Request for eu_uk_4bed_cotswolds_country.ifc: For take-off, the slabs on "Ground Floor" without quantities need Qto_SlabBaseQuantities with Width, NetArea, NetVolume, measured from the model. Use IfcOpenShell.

First a look at what the model holds.

```python
import ifcopenshell
import ifcopenshell.util.element
import ifcopenshell.util.unit

model = ifcopenshell.open("eu_uk_4bed_cotswolds_country.ifc")
print(model.schema)
for unit_type in ("LENGTHUNIT", "AREAUNIT", "VOLUMEUNIT"):
    print(unit_type, ifcopenshell.util.unit.calculate_unit_scale(model, unit_type))
storey = next(s for s in model.by_type("IfcBuildingStorey") if s.Name == "Ground Floor")
slabs = [e for e in ifcopenshell.util.element.get_decomposition(storey) if e.is_a("IfcSlab")]
for e in sorted(slabs, key=lambda e: e.id()):
    print(e.id(), e.is_a(), e.Name, list(ifcopenshell.util.element.get_psets(e, qtos_only=True)), sep=" | ")
```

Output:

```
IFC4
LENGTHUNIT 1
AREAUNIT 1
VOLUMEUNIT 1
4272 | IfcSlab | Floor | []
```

```python
import ifcopenshell
import ifcopenshell.api.pset
import ifcopenshell.geom
import ifcopenshell.util.element
import ifcopenshell.util.shape
import ifcopenshell.util.unit

model = ifcopenshell.open("eu_uk_4bed_cotswolds_country.ifc")
unit_scale = ifcopenshell.util.unit.calculate_unit_scale(model)
area_scale = ifcopenshell.util.unit.calculate_unit_scale(model, "AREAUNIT")
volume_scale = ifcopenshell.util.unit.calculate_unit_scale(model, "VOLUMEUNIT")
settings = ifcopenshell.geom.settings()

storey = next(s for s in model.by_type("IfcBuildingStorey") if s.Name == "Ground Floor")
slabs = [e for e in ifcopenshell.util.element.get_decomposition(storey) if e.is_a("IfcSlab")]

for e in sorted(slabs, key=lambda e: e.id()):
    if ifcopenshell.util.element.get_psets(e, qtos_only=True, should_inherit=False):
        continue
    # Geometry comes back in metres, in the element's own axes.
    shape = ifcopenshell.geom.create_shape(settings, e)
    values = {
        "Width": ifcopenshell.util.shape.get_z(shape.geometry) / unit_scale,
        "NetArea": ifcopenshell.util.shape.get_footprint_area(shape.geometry) / area_scale,
        "NetVolume": ifcopenshell.util.shape.get_volume(shape.geometry) / volume_scale,
    }
    qto = ifcopenshell.api.pset.add_qto(model, product=e, name="Qto_SlabBaseQuantities")
    ifcopenshell.api.pset.edit_qto(model, qto=qto, properties=values)
    print(e.id(), {k: round(v, 3) for k, v in values.items()})

model.write("eu_uk_4bed_cotswolds_country_v2.ifc")
```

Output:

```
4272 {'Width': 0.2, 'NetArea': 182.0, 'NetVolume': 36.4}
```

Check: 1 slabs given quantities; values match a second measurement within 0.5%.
